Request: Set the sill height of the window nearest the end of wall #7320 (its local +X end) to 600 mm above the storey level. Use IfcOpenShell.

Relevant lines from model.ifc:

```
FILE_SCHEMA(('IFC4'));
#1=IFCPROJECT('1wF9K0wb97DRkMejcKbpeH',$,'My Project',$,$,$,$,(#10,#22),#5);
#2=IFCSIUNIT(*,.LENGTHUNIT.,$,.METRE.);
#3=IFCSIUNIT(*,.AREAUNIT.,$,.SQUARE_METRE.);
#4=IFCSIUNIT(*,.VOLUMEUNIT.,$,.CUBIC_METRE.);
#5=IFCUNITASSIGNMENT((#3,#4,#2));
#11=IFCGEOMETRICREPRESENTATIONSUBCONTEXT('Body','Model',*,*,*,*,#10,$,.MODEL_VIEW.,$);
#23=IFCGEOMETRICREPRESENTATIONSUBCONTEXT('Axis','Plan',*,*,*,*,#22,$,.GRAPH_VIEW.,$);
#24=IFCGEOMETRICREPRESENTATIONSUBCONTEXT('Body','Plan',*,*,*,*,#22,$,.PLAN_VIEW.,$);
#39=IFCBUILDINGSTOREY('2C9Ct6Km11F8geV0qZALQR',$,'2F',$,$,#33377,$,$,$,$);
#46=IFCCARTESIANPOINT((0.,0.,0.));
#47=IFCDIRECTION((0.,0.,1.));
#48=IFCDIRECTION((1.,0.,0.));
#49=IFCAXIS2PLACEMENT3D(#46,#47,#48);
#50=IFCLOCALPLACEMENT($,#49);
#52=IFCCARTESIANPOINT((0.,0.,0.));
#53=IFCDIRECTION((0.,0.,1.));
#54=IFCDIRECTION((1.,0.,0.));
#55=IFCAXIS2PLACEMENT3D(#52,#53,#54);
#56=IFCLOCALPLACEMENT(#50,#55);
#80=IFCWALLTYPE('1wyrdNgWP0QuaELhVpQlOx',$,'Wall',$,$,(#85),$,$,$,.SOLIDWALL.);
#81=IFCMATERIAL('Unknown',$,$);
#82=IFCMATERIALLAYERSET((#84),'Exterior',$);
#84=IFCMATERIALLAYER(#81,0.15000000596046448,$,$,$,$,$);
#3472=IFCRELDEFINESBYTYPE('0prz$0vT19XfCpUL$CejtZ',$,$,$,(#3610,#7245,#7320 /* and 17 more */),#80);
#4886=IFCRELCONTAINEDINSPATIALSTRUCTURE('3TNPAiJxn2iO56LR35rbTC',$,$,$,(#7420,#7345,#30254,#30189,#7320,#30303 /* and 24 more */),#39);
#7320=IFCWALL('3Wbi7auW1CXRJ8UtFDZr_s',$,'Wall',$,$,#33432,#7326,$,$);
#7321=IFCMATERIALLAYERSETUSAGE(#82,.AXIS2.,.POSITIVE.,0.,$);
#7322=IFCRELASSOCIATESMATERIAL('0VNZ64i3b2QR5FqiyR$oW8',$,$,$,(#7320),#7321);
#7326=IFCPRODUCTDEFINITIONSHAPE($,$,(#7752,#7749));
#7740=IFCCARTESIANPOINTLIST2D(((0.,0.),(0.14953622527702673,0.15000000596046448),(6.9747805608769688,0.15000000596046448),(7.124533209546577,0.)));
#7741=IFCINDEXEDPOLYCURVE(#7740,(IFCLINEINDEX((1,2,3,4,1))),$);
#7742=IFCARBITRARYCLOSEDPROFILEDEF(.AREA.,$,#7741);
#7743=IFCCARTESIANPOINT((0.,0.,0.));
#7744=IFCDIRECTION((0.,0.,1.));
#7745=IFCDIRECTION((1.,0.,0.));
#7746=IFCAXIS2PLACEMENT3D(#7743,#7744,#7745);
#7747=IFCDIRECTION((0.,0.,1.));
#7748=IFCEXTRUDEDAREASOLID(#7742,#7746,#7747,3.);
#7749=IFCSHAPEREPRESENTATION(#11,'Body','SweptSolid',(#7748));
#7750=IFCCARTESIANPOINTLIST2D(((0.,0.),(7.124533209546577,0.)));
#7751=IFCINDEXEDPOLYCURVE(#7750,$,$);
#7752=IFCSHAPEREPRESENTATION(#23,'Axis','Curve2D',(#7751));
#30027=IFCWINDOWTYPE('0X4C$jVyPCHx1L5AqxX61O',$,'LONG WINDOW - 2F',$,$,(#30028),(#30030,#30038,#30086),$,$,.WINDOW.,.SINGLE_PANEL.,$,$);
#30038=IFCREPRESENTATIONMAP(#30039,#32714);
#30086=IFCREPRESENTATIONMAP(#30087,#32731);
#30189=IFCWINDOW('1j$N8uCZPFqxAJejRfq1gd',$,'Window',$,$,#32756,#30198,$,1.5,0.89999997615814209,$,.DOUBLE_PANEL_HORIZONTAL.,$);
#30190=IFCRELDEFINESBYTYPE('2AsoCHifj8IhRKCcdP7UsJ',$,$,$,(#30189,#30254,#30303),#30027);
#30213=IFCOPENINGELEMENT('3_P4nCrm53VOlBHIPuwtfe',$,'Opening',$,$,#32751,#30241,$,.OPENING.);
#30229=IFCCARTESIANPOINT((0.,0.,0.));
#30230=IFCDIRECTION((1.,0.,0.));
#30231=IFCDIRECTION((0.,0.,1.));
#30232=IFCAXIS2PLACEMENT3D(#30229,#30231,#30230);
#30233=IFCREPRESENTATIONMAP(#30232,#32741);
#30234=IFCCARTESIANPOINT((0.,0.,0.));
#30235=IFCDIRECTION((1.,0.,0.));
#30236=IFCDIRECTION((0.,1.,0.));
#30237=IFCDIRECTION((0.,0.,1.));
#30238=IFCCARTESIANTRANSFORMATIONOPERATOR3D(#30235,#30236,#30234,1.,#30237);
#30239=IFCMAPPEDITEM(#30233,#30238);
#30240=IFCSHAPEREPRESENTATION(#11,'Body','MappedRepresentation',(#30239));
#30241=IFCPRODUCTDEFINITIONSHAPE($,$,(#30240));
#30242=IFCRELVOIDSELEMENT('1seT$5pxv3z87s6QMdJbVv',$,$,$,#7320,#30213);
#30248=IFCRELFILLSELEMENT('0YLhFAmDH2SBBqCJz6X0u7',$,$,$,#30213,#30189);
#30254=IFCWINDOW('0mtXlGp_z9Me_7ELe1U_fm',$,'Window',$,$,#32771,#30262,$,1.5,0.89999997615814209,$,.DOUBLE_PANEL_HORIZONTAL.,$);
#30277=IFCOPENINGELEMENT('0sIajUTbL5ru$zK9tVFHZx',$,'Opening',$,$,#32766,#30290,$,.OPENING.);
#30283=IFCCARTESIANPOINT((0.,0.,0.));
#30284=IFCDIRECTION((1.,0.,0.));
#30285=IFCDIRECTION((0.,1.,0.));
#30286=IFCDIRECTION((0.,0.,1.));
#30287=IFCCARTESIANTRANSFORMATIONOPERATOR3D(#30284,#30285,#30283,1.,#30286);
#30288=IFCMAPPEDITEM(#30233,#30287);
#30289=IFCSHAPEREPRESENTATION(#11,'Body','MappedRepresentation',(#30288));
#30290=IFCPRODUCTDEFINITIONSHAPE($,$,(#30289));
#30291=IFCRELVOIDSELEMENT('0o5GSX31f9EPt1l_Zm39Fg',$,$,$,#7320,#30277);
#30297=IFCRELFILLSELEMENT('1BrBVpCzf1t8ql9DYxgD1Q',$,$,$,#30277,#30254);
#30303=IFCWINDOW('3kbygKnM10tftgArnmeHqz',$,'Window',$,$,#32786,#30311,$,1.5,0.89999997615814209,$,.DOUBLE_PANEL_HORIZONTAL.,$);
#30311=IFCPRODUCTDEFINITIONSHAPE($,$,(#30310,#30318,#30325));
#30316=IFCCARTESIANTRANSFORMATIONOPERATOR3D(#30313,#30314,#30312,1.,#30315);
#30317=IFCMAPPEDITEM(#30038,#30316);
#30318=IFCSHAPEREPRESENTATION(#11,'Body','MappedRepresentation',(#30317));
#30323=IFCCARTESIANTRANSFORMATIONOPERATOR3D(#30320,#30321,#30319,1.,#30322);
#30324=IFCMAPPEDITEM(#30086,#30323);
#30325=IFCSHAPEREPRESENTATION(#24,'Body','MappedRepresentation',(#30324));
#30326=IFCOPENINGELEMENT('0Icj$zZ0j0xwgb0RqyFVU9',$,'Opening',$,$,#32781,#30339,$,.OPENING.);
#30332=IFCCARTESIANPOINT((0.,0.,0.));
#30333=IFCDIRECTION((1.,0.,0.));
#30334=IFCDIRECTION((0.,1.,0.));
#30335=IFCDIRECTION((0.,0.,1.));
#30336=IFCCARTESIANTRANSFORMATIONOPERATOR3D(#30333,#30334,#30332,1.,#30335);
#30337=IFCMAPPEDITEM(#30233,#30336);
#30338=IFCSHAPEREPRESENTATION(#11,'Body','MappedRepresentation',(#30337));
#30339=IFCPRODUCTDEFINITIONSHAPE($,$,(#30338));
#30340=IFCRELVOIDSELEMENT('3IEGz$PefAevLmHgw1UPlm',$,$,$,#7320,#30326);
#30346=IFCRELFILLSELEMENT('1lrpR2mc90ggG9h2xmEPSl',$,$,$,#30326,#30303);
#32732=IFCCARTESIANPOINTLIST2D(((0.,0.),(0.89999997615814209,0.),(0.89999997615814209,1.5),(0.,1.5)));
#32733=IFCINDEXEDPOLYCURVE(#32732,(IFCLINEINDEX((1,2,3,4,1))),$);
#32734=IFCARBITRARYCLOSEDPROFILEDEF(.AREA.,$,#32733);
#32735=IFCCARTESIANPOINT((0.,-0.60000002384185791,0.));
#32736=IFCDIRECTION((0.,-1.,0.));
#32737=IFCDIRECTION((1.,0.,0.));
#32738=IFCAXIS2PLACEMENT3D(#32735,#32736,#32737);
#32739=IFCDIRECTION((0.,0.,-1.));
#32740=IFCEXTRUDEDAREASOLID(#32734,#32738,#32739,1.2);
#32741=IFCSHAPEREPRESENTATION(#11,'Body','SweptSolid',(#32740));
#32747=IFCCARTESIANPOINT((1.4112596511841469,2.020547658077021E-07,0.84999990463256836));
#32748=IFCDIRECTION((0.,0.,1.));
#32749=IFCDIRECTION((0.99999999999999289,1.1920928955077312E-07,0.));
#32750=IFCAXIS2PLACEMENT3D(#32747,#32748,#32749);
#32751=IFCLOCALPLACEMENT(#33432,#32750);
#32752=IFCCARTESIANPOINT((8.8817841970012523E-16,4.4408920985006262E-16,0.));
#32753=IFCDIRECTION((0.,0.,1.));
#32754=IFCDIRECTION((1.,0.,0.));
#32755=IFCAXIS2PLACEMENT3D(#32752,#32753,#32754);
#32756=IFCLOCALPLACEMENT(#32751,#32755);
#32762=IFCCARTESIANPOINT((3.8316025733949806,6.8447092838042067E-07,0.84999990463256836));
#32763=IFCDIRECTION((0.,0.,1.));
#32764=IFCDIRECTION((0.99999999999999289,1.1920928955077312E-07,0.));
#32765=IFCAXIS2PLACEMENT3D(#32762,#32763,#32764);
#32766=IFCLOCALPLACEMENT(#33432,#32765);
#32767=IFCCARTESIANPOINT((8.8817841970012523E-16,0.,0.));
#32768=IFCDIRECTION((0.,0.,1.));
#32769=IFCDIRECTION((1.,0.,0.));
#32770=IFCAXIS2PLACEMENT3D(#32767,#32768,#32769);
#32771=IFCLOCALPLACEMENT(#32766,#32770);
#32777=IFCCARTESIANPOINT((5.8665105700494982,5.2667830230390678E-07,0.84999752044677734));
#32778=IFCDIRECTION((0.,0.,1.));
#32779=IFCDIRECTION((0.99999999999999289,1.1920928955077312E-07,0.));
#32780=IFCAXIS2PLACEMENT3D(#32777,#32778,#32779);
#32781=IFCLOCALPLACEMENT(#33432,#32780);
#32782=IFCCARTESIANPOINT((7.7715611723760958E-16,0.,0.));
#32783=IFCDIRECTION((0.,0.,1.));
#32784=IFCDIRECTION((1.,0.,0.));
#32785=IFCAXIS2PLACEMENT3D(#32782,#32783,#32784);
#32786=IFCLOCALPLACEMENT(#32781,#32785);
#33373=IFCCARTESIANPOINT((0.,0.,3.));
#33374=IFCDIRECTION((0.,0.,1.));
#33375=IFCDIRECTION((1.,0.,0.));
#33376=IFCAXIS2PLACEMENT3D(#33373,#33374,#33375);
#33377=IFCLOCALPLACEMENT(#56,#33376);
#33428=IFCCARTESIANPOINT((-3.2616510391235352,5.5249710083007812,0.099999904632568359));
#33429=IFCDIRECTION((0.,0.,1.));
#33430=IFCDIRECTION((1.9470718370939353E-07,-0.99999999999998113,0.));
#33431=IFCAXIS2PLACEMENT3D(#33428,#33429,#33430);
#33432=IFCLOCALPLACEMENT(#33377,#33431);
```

```python
import numpy as np
import ifcopenshell
import ifcopenshell.api.geometry
import ifcopenshell.geom
import ifcopenshell.util.element
import ifcopenshell.util.placement
import ifcopenshell.util.shape
import ifcopenshell.util.unit

model = ifcopenshell.open("model.ifc")
unit_scale = ifcopenshell.util.unit.calculate_unit_scale(model)

window = model.by_guid("3kbygKnM10tftgArnmeHqz")
opening = window.FillsVoids[0].RelatingOpeningElement
storey = ifcopenshell.util.element.get_container(window, ifc_class="IfcBuildingStorey")
level = ifcopenshell.util.placement.get_local_placement(storey.ObjectPlacement)[2, 3]

# The opening's origin need not be at the sill, so measure its lowest point.
shape = ifcopenshell.geom.create_shape(ifcopenshell.geom.settings(), opening)
bottom = ifcopenshell.util.shape.get_shape_bottom_elevation(shape, shape.geometry) / unit_scale
dz = level + 0.6 / unit_scale - bottom

shift = np.array([0.0, 0.0, dz])
# The window is placed relative to its opening, so it follows when the opening moves.
matrix = ifcopenshell.util.placement.get_local_placement(opening.ObjectPlacement)
matrix[:3, 3] += shift
ifcopenshell.api.geometry.edit_object_placement(
    model, product=opening, matrix=matrix, is_si=False, should_transform_children=True
)

print(f"moved by {dz * unit_scale:+.3f} m")

model.write("model_edited.ifc")
```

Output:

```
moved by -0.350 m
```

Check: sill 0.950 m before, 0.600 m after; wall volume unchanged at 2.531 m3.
